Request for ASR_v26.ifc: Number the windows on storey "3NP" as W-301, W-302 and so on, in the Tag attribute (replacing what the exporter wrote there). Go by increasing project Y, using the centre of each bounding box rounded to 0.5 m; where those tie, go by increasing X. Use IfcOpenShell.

First a look at what the model holds.

```python
import ifcopenshell
import ifcopenshell.util.element
import ifcopenshell.util.placement

model = ifcopenshell.open("ASR_v26.ifc")
print(model.schema)
storey = next(s for s in model.by_type("IfcBuildingStorey") if s.Name == "3NP")
windows = [e for e in ifcopenshell.util.element.get_decomposition(storey) if e.is_a("IfcWindow")]
for e in sorted(windows, key=lambda e: e.id()):
    origin = ifcopenshell.util.placement.get_local_placement(e.ObjectPlacement)[:3, 3]
    print(e.id(), e.Tag, e.Name, origin.round(2) + 0.0, sep=" | ")
```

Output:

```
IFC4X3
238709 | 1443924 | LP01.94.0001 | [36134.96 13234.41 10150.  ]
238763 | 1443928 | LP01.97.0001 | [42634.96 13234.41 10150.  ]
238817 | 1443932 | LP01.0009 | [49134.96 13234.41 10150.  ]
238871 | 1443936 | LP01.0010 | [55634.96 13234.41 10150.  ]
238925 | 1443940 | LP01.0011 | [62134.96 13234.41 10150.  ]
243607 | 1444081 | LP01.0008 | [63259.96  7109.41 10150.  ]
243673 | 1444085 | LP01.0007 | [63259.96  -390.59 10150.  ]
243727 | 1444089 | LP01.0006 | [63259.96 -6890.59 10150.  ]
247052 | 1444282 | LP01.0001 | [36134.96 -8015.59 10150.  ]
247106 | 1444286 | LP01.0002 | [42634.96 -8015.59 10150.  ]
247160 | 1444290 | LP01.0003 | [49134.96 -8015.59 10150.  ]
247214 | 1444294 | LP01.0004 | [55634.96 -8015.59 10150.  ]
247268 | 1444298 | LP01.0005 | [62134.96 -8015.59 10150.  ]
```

```python
import ifcopenshell
import ifcopenshell.geom
import ifcopenshell.util.element
import ifcopenshell.util.shape

model = ifcopenshell.open("ASR_v26.ifc")
settings = ifcopenshell.geom.settings()
settings.set("use-world-coords", True)


def centre(element):
    shape = ifcopenshell.geom.create_shape(settings, element)
    return ifcopenshell.util.shape.get_bbox_centroid(shape.geometry)


storey = next(s for s in model.by_type("IfcBuildingStorey") if s.Name == "3NP")
windows = [e for e in ifcopenshell.util.element.get_decomposition(storey) if e.is_a("IfcWindow")]

# Insertion points can sit at a corner or the storey origin, so sort by the geometry (in metres).
centres = {e: centre(e) for e in windows}
windows.sort(key=lambda e: (round(centres[e][1] / 0.5), centres[e][0]))

for i, e in enumerate(windows, start=1):
    number = f"W-3{i:02d}"
    e.Tag = number
    print(e.id(), number)

model.write("ASR_v26_v2.ifc")
```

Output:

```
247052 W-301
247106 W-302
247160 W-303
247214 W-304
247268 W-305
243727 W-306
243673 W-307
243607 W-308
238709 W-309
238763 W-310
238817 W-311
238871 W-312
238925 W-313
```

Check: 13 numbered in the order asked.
